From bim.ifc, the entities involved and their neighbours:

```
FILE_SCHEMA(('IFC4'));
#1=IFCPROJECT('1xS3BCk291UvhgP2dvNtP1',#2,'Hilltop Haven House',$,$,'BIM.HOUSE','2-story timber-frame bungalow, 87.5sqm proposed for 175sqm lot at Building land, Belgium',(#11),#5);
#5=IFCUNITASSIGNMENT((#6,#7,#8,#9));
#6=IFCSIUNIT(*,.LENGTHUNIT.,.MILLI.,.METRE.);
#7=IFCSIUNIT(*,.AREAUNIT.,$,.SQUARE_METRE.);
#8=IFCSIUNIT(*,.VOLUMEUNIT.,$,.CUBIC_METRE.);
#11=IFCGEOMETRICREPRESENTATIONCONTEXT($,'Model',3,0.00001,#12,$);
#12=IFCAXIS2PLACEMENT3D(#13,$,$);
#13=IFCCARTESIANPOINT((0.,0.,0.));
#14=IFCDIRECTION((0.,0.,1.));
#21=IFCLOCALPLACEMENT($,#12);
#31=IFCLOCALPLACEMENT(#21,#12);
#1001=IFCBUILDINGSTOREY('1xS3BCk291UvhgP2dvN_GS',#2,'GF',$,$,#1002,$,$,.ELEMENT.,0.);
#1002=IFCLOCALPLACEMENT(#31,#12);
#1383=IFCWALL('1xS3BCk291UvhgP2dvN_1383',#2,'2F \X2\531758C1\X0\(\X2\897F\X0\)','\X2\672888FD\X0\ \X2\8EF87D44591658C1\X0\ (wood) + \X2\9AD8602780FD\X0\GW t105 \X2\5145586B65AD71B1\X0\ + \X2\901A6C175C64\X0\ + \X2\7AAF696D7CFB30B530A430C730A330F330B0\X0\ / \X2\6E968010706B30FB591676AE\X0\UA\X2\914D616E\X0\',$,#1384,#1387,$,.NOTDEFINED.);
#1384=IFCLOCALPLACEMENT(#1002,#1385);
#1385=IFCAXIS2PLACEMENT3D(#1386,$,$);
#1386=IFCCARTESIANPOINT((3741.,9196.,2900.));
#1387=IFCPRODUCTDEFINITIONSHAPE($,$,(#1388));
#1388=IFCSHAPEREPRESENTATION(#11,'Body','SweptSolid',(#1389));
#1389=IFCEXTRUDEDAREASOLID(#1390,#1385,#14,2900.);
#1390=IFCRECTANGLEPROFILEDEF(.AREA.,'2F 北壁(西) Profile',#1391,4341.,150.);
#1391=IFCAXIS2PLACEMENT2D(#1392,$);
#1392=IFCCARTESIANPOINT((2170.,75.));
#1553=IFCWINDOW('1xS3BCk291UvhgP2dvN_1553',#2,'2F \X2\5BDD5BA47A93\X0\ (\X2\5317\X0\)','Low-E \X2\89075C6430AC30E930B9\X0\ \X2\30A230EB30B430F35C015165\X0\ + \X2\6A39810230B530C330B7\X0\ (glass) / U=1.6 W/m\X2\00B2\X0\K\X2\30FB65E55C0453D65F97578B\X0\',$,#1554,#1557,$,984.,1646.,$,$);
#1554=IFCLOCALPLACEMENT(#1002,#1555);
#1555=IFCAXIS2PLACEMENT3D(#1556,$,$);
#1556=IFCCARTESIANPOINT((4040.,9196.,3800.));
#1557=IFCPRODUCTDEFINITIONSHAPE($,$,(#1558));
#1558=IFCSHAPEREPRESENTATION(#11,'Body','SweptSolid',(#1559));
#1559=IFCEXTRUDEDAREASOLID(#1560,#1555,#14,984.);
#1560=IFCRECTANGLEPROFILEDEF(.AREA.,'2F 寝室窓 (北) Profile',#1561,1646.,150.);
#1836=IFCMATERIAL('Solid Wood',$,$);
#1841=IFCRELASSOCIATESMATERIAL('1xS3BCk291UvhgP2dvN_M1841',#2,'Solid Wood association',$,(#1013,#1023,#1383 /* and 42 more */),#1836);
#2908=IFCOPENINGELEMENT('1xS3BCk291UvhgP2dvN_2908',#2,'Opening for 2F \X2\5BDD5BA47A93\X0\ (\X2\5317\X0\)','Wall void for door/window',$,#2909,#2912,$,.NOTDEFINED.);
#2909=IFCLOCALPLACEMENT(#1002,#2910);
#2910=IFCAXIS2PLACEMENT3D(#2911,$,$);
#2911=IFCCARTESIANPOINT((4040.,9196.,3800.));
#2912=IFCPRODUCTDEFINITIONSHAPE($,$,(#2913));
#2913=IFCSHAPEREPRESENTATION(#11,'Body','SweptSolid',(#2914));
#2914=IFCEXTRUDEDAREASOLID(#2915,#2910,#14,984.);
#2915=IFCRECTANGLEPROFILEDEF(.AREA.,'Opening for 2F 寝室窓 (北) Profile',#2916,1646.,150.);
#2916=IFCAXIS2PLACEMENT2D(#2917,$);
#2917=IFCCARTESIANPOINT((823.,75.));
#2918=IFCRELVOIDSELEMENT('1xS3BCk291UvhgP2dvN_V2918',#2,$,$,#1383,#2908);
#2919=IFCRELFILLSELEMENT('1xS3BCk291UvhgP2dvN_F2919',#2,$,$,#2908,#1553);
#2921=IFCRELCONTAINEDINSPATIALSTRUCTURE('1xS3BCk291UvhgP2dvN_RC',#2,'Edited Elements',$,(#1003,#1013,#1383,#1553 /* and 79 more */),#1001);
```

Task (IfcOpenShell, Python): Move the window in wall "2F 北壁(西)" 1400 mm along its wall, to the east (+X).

```python
import ifcopenshell
import ifcopenshell.api.geometry
import ifcopenshell.util.placement
import ifcopenshell.util.unit

model = ifcopenshell.open("bim.ifc")
unit_scale = ifcopenshell.util.unit.calculate_unit_scale(model)

window = model.by_id(1553)
opening = window.FillsVoids[0].RelatingOpeningElement
wall = opening.VoidsElements[0].RelatingBuildingElement

wall_matrix = ifcopenshell.util.placement.get_local_placement(wall.ObjectPlacement)
shift = wall_matrix[:3, 0] * 1.4 / unit_scale
before = ifcopenshell.util.placement.get_local_placement(window.ObjectPlacement)[:3, 3].copy()

# The window is not placed relative to its opening, so move both.
for product in (opening, window):
    matrix = ifcopenshell.util.placement.get_local_placement(product.ObjectPlacement)
    matrix[:3, 3] += shift
    ifcopenshell.api.geometry.edit_object_placement(model, product=product, matrix=matrix, is_si=False)

after = ifcopenshell.util.placement.get_local_placement(window.ObjectPlacement)[:3, 3]
print("window moved by", (after - before).round(3) + 0.0)

model.write("bim-out.ifc")
```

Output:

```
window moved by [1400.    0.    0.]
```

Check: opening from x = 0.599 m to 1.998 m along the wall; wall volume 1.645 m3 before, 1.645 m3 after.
